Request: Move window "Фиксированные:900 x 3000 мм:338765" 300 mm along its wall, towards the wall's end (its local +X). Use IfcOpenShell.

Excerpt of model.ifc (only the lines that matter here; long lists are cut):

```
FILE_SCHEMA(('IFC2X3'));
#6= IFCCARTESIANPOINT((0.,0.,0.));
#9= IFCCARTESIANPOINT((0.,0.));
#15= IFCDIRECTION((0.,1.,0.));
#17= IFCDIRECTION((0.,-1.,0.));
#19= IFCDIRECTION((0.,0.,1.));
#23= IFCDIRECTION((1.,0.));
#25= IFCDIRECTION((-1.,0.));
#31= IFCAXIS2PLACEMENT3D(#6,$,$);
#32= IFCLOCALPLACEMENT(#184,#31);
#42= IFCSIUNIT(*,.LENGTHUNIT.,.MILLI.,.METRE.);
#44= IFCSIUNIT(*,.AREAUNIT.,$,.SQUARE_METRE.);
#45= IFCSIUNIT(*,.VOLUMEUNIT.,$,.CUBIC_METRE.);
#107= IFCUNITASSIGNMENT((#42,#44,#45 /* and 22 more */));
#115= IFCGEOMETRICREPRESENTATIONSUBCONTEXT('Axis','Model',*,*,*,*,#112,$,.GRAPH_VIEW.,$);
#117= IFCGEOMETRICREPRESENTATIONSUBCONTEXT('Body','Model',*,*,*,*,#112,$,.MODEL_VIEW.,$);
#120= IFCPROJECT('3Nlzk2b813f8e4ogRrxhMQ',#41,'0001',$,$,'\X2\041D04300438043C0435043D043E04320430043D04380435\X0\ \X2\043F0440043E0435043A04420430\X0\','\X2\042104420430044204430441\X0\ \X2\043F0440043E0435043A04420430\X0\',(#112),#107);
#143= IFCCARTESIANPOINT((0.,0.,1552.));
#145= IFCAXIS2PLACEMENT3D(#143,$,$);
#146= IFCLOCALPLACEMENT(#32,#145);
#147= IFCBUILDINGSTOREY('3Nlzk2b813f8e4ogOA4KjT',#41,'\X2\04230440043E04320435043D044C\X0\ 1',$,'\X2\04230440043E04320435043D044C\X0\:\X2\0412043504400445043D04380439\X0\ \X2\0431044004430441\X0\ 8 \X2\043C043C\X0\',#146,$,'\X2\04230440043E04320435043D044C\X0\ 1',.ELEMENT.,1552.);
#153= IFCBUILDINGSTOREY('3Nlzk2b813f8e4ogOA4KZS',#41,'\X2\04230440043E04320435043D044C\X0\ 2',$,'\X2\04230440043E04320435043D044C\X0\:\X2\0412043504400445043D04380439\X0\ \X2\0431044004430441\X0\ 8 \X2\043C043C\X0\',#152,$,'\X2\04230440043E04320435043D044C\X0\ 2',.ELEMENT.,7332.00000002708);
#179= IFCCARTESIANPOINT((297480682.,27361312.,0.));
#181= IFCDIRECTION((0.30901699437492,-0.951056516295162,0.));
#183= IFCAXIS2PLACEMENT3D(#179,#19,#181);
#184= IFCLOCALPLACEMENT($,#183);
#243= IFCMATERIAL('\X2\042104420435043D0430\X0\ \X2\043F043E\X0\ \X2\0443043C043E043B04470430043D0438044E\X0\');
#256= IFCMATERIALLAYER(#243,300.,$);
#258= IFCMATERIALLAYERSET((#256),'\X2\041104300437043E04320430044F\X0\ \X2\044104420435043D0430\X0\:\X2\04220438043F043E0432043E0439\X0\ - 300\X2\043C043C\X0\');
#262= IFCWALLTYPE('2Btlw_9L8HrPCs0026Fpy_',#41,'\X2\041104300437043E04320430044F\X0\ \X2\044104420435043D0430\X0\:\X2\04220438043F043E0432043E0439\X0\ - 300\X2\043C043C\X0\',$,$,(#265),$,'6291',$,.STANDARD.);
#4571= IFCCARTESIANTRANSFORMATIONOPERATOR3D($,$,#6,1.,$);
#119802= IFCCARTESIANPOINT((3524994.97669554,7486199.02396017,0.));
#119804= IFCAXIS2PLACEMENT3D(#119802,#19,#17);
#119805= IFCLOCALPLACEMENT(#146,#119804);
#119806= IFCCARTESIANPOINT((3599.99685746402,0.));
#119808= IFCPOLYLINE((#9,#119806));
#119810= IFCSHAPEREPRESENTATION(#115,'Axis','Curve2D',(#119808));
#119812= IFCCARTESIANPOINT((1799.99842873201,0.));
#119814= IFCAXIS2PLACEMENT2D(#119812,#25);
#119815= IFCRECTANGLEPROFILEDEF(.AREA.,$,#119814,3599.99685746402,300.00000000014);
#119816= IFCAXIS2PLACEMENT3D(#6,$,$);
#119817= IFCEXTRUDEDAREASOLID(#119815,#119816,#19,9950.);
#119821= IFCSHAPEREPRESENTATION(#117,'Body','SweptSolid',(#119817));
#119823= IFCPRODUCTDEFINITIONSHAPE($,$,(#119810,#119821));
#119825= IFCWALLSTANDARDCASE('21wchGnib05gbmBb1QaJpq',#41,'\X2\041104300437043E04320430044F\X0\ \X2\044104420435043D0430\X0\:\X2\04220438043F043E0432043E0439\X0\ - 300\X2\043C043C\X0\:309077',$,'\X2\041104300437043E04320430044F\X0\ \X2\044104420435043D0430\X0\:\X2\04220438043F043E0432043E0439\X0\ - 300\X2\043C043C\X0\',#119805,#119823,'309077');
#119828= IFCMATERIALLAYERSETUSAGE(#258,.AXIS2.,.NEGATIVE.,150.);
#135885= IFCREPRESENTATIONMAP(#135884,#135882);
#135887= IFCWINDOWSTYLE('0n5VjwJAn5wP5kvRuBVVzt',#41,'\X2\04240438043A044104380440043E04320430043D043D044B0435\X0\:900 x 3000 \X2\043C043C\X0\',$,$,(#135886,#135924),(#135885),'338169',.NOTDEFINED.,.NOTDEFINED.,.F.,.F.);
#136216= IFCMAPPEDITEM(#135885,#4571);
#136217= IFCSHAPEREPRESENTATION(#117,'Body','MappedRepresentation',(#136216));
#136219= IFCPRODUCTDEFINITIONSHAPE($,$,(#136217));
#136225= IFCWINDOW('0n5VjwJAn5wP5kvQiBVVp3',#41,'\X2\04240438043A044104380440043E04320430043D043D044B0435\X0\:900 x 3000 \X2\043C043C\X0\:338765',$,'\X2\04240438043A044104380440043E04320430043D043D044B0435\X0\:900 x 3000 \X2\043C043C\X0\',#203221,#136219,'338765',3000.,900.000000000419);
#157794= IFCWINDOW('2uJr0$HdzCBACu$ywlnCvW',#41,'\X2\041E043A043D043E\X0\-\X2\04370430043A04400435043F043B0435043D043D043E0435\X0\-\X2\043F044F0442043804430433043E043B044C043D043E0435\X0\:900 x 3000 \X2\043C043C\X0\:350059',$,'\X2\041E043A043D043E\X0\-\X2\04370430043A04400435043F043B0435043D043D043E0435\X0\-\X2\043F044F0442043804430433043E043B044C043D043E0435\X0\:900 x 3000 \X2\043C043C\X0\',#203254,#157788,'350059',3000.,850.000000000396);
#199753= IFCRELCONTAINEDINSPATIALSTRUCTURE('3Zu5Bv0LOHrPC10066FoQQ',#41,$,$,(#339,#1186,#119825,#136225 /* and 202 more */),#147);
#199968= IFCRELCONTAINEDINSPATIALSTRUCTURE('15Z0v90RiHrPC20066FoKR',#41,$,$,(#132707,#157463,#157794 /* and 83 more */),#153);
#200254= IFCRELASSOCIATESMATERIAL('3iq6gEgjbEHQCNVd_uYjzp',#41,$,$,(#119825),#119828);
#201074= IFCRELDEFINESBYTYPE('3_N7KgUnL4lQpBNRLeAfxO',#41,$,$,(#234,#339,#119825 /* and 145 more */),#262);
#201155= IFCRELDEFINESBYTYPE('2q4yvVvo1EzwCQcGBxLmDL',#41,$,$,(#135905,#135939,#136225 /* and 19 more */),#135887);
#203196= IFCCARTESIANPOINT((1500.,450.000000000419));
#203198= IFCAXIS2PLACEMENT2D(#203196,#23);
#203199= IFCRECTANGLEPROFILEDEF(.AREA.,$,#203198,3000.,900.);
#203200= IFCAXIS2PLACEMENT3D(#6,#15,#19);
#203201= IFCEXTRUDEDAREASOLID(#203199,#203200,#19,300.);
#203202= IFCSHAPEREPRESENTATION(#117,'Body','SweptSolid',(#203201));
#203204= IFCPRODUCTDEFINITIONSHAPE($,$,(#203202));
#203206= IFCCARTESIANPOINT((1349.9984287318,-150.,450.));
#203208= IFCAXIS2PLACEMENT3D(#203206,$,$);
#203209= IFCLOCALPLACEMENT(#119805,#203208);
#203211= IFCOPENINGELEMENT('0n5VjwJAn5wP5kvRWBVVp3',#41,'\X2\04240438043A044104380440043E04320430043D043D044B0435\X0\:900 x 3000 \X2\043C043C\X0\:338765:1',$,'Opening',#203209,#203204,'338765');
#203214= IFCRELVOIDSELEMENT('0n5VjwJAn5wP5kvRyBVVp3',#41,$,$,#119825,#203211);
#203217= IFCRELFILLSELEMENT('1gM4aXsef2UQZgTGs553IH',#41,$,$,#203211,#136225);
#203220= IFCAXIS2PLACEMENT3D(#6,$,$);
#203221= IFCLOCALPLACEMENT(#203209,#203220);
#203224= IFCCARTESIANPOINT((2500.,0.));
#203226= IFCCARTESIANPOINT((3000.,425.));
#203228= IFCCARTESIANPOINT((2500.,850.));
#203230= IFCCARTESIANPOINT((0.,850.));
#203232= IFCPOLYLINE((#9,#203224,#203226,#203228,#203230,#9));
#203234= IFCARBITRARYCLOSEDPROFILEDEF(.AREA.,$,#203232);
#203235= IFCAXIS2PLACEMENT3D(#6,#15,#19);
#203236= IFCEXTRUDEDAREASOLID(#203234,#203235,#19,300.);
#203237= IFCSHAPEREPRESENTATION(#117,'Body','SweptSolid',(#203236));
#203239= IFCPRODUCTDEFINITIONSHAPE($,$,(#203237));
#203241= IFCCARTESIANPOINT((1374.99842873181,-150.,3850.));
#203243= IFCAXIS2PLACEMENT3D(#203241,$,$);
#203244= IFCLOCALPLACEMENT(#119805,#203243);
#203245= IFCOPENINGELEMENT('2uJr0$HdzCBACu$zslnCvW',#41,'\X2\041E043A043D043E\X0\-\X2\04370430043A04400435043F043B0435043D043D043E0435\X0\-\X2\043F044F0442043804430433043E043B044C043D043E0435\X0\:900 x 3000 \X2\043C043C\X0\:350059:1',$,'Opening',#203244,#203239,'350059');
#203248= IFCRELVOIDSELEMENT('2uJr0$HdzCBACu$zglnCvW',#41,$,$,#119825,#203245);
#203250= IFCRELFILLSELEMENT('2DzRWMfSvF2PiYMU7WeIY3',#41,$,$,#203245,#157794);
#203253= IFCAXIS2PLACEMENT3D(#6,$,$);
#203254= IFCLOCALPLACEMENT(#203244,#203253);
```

```python
import ifcopenshell
import ifcopenshell.api.geometry
import ifcopenshell.util.placement
import ifcopenshell.util.unit

model = ifcopenshell.open("model.ifc")
unit_scale = ifcopenshell.util.unit.calculate_unit_scale(model)

window = model.by_guid("0n5VjwJAn5wP5kvQiBVVp3")
opening = window.FillsVoids[0].RelatingOpeningElement
wall = opening.VoidsElements[0].RelatingBuildingElement

wall_matrix = ifcopenshell.util.placement.get_local_placement(wall.ObjectPlacement)
shift = wall_matrix[:3, 0] * 0.3 / unit_scale
before = ifcopenshell.util.placement.get_local_placement(window.ObjectPlacement)[:3, 3].copy()

# The window is placed relative to its opening, so it follows when the opening moves.
matrix = ifcopenshell.util.placement.get_local_placement(opening.ObjectPlacement)
matrix[:3, 3] += shift
ifcopenshell.api.geometry.edit_object_placement(
    model, product=opening, matrix=matrix, is_si=False, should_transform_children=True
)

after = ifcopenshell.util.placement.get_local_placement(window.ObjectPlacement)[:3, 3]
print("window moved by", (after - before).round(3) + 0.0)

model.write("model_updated.ifc")
```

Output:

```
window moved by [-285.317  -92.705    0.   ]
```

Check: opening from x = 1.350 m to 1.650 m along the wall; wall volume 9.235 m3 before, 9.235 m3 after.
